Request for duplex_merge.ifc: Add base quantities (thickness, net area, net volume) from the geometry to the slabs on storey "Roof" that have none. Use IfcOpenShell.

First a look at what the model holds.

```python
import ifcopenshell
import ifcopenshell.util.element
import ifcopenshell.util.unit

model = ifcopenshell.open("duplex_merge.ifc")
print(model.schema)
for unit_type in ("LENGTHUNIT", "AREAUNIT", "VOLUMEUNIT"):
    print(unit_type, ifcopenshell.util.unit.calculate_unit_scale(model, unit_type))
storey = next(s for s in model.by_type("IfcBuildingStorey") if s.Name == "Roof")
slabs = [e for e in ifcopenshell.util.element.get_decomposition(storey) if e.is_a("IfcSlab")]
for e in sorted(slabs, key=lambda e: e.id()):
    print(e.id(), e.is_a(), e.Name, list(ifcopenshell.util.element.get_psets(e, qtos_only=True)), sep=" | ")
```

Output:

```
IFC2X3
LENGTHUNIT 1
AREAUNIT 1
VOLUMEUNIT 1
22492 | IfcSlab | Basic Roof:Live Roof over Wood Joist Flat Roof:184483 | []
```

```python
import ifcopenshell
import ifcopenshell.api.pset
import ifcopenshell.geom
import ifcopenshell.util.element
import ifcopenshell.util.shape
import ifcopenshell.util.unit

model = ifcopenshell.open("duplex_merge.ifc")
unit_scale = ifcopenshell.util.unit.calculate_unit_scale(model)
area_scale = ifcopenshell.util.unit.calculate_unit_scale(model, "AREAUNIT")
volume_scale = ifcopenshell.util.unit.calculate_unit_scale(model, "VOLUMEUNIT")
settings = ifcopenshell.geom.settings()

storey = next(s for s in model.by_type("IfcBuildingStorey") if s.Name == "Roof")
slabs = [e for e in ifcopenshell.util.element.get_decomposition(storey) if e.is_a("IfcSlab")]

for e in sorted(slabs, key=lambda e: e.id()):
    if ifcopenshell.util.element.get_psets(e, qtos_only=True, should_inherit=False):
        continue
    # Geometry comes back in metres, in the element's own axes.
    shape = ifcopenshell.geom.create_shape(settings, e)
    values = {
        "Width": ifcopenshell.util.shape.get_z(shape.geometry) / unit_scale,
        "NetArea": ifcopenshell.util.shape.get_footprint_area(shape.geometry) / area_scale,
        "NetVolume": ifcopenshell.util.shape.get_volume(shape.geometry) / volume_scale,
    }
    qto = ifcopenshell.api.pset.add_qto(model, product=e, name="BaseQuantities")
    ifcopenshell.api.pset.edit_qto(model, qto=qto, properties=values)
    print(e.id(), {k: round(v, 3) for k, v in values.items()})

model.write("duplex_merge_edited.ifc")
```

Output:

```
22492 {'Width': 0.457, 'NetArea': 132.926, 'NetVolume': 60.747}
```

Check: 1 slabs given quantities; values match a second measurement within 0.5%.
